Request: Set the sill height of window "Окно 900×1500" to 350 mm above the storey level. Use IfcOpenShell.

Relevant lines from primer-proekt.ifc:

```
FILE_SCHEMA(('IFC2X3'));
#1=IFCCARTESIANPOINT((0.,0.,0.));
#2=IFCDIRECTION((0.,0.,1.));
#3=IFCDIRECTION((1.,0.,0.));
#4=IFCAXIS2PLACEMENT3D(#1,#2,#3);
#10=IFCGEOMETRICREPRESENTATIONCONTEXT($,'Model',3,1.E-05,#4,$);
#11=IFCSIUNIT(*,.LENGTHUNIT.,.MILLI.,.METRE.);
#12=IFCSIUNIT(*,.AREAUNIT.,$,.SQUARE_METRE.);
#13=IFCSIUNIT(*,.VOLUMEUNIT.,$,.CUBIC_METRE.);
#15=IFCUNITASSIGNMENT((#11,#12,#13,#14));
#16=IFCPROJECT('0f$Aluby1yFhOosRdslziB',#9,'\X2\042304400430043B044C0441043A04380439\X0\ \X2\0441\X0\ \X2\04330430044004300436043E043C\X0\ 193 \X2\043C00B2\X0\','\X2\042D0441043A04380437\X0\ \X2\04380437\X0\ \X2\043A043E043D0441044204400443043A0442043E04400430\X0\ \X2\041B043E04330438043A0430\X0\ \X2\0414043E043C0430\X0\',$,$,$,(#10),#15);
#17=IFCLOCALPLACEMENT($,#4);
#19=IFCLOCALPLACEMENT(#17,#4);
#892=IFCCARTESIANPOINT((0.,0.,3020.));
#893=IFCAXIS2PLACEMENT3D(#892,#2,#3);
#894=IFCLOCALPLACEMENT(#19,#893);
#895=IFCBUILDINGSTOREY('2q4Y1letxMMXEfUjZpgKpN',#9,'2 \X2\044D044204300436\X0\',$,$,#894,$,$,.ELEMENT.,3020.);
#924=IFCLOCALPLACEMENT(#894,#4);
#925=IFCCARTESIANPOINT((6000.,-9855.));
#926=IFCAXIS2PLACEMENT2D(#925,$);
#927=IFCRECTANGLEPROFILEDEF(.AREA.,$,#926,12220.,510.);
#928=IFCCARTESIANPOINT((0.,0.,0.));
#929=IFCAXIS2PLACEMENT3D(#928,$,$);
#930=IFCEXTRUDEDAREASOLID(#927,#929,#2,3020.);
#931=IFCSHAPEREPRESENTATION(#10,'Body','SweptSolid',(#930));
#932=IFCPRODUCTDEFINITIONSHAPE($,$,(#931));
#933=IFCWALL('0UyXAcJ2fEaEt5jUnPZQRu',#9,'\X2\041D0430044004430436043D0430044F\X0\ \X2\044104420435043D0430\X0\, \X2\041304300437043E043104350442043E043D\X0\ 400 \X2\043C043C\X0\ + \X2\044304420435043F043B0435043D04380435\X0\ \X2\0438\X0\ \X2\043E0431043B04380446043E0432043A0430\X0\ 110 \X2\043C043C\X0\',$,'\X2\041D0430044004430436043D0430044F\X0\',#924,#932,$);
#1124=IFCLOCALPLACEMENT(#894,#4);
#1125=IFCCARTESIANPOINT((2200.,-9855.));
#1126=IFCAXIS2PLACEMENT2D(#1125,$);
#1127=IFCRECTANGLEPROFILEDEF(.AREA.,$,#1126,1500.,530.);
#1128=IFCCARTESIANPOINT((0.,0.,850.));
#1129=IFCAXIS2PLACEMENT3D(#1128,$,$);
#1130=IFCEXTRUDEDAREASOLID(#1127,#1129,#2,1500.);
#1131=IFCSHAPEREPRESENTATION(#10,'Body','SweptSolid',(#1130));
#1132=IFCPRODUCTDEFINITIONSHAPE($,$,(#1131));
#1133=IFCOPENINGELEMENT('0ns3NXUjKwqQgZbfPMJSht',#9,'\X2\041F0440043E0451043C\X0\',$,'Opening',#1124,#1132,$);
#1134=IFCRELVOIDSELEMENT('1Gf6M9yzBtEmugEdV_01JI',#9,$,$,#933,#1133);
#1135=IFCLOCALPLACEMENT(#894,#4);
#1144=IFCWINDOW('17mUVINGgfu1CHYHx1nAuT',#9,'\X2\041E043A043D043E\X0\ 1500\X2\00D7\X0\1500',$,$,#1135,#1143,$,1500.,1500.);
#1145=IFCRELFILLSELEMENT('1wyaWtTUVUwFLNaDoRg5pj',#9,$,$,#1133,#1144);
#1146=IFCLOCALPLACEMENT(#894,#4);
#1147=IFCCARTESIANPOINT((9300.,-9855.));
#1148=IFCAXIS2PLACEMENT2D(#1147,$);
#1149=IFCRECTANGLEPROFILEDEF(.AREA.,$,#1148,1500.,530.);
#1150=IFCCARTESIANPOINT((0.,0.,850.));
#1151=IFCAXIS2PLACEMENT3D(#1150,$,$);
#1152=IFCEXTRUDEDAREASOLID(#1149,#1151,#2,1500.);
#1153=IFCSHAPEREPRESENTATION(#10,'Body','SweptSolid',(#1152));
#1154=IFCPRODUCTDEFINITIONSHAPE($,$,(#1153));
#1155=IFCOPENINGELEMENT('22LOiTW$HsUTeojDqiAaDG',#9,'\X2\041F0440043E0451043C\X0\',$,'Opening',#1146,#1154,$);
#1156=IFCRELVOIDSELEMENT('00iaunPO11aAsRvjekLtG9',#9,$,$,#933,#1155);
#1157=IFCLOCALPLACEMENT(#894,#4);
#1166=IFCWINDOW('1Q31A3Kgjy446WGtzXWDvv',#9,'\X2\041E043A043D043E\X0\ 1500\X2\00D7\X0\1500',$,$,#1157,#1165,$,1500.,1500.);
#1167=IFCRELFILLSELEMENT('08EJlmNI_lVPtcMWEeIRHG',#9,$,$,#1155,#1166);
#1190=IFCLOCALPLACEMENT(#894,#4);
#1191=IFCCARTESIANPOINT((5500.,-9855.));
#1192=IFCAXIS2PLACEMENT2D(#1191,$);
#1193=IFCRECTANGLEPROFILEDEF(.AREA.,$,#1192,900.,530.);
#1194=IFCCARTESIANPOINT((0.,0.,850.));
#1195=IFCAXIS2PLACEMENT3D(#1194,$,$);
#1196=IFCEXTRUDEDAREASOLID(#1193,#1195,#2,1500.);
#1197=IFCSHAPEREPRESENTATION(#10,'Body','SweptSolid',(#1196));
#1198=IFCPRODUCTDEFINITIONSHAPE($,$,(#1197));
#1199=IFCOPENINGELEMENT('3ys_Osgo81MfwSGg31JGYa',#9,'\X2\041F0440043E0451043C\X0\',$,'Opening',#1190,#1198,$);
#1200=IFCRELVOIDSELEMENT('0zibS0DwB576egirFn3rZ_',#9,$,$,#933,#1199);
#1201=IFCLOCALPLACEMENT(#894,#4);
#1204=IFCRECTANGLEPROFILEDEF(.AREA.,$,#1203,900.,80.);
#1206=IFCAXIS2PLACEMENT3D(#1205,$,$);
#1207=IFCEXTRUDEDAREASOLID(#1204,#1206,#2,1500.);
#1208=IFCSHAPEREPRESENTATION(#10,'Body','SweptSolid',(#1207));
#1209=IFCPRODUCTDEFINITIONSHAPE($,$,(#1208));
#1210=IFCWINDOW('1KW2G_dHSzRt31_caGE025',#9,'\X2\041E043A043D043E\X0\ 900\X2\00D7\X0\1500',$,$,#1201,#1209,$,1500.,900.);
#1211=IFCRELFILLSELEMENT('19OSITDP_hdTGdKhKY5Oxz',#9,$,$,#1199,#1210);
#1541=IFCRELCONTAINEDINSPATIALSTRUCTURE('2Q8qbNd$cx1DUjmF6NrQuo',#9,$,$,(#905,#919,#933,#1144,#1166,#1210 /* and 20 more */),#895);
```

```python
import numpy as np
import ifcopenshell
import ifcopenshell.api.geometry
import ifcopenshell.geom
import ifcopenshell.util.element
import ifcopenshell.util.placement
import ifcopenshell.util.shape
import ifcopenshell.util.unit

model = ifcopenshell.open("primer-proekt.ifc")
unit_scale = ifcopenshell.util.unit.calculate_unit_scale(model)

window = model.by_guid("1KW2G_dHSzRt31_caGE025")
opening = window.FillsVoids[0].RelatingOpeningElement
storey = ifcopenshell.util.element.get_container(window, ifc_class="IfcBuildingStorey")
level = ifcopenshell.util.placement.get_local_placement(storey.ObjectPlacement)[2, 3]

# The opening's origin need not be at the sill, so measure its lowest point.
shape = ifcopenshell.geom.create_shape(ifcopenshell.geom.settings(), opening)
bottom = ifcopenshell.util.shape.get_shape_bottom_elevation(shape, shape.geometry) / unit_scale
dz = level + 0.35 / unit_scale - bottom

shift = np.array([0.0, 0.0, dz])
# The window is not placed relative to its opening, so move both.
for product in (opening, window):
    matrix = ifcopenshell.util.placement.get_local_placement(product.ObjectPlacement)
    matrix[:3, 3] += shift
    ifcopenshell.api.geometry.edit_object_placement(model, product=product, matrix=matrix, is_si=False)

print(f"moved by {dz * unit_scale:+.3f} m")

model.write("primer-proekt_updated.ifc")
```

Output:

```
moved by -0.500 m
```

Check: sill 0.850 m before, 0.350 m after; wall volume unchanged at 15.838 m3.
